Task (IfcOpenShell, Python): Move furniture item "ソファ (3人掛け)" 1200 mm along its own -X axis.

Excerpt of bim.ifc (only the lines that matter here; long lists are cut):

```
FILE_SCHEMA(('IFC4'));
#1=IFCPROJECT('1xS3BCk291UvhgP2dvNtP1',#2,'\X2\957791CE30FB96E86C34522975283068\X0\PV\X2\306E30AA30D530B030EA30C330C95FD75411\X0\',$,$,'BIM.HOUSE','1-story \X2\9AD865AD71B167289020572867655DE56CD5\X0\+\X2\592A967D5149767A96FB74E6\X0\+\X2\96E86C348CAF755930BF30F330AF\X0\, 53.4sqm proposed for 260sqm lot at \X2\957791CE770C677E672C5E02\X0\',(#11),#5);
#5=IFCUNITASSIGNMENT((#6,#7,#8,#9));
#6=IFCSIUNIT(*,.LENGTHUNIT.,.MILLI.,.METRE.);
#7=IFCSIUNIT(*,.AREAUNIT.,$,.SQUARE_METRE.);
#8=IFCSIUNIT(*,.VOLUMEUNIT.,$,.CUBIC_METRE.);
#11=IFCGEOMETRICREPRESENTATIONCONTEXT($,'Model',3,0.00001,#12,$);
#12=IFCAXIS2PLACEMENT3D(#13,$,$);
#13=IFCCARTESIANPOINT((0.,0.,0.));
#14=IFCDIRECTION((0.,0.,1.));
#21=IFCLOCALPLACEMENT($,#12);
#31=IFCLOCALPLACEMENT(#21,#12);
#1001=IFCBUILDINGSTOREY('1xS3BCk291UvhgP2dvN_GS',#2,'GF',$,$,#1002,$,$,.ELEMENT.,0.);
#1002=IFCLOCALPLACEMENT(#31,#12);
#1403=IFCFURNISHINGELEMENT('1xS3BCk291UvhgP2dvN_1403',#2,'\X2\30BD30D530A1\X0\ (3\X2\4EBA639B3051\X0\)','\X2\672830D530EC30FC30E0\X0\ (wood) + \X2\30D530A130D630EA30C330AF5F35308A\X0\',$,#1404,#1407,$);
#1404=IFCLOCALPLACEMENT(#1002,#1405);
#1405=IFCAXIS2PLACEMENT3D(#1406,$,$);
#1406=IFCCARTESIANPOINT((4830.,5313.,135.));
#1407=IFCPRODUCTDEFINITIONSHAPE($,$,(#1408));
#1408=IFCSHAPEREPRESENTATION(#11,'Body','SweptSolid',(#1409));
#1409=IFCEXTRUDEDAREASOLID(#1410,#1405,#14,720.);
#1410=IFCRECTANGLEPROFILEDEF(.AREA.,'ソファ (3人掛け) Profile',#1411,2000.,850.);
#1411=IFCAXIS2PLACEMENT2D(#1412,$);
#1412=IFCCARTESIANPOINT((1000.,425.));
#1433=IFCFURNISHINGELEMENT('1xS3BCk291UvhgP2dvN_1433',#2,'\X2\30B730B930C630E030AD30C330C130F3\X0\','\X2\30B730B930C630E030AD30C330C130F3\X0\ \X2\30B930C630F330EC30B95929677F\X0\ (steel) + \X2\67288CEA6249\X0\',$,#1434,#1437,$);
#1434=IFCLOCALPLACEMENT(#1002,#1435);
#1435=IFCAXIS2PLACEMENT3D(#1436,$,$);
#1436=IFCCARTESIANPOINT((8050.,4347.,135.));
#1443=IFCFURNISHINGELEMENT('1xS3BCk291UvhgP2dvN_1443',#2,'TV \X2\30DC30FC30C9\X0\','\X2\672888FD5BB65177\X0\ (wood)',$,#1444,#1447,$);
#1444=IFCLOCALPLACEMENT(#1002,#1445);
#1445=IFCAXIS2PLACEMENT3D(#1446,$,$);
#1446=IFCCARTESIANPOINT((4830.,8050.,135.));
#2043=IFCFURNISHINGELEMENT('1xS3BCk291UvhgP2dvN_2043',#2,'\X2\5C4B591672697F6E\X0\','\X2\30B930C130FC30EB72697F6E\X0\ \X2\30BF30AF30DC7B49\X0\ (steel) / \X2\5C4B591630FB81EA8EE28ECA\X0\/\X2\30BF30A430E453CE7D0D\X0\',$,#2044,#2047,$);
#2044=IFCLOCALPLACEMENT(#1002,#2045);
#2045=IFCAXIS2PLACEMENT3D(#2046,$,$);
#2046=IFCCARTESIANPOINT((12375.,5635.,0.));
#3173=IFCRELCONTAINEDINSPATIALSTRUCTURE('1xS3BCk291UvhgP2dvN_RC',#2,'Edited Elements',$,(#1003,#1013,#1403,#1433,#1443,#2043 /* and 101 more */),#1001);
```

```python
import ifcopenshell
import ifcopenshell.api.geometry
import ifcopenshell.util.placement
import ifcopenshell.util.unit

model = ifcopenshell.open("bim.ifc")
unit_scale = ifcopenshell.util.unit.calculate_unit_scale(model)

item = model.by_guid("1xS3BCk291UvhgP2dvN_1403")
matrix = ifcopenshell.util.placement.get_local_placement(item.ObjectPlacement)
matrix[:3, 3] -= matrix[:3, 0] * 1.2 / unit_scale
ifcopenshell.api.geometry.edit_object_placement(model, product=item, matrix=matrix, is_si=False)

print(ifcopenshell.util.placement.get_local_placement(item.ObjectPlacement).round(3) + 0.0)

model.write("bim_updated.ifc")
```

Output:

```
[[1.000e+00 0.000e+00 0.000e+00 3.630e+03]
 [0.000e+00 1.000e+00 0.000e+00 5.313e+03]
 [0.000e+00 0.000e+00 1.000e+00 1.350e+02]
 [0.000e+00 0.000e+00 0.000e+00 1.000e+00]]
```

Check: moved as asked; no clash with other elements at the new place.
